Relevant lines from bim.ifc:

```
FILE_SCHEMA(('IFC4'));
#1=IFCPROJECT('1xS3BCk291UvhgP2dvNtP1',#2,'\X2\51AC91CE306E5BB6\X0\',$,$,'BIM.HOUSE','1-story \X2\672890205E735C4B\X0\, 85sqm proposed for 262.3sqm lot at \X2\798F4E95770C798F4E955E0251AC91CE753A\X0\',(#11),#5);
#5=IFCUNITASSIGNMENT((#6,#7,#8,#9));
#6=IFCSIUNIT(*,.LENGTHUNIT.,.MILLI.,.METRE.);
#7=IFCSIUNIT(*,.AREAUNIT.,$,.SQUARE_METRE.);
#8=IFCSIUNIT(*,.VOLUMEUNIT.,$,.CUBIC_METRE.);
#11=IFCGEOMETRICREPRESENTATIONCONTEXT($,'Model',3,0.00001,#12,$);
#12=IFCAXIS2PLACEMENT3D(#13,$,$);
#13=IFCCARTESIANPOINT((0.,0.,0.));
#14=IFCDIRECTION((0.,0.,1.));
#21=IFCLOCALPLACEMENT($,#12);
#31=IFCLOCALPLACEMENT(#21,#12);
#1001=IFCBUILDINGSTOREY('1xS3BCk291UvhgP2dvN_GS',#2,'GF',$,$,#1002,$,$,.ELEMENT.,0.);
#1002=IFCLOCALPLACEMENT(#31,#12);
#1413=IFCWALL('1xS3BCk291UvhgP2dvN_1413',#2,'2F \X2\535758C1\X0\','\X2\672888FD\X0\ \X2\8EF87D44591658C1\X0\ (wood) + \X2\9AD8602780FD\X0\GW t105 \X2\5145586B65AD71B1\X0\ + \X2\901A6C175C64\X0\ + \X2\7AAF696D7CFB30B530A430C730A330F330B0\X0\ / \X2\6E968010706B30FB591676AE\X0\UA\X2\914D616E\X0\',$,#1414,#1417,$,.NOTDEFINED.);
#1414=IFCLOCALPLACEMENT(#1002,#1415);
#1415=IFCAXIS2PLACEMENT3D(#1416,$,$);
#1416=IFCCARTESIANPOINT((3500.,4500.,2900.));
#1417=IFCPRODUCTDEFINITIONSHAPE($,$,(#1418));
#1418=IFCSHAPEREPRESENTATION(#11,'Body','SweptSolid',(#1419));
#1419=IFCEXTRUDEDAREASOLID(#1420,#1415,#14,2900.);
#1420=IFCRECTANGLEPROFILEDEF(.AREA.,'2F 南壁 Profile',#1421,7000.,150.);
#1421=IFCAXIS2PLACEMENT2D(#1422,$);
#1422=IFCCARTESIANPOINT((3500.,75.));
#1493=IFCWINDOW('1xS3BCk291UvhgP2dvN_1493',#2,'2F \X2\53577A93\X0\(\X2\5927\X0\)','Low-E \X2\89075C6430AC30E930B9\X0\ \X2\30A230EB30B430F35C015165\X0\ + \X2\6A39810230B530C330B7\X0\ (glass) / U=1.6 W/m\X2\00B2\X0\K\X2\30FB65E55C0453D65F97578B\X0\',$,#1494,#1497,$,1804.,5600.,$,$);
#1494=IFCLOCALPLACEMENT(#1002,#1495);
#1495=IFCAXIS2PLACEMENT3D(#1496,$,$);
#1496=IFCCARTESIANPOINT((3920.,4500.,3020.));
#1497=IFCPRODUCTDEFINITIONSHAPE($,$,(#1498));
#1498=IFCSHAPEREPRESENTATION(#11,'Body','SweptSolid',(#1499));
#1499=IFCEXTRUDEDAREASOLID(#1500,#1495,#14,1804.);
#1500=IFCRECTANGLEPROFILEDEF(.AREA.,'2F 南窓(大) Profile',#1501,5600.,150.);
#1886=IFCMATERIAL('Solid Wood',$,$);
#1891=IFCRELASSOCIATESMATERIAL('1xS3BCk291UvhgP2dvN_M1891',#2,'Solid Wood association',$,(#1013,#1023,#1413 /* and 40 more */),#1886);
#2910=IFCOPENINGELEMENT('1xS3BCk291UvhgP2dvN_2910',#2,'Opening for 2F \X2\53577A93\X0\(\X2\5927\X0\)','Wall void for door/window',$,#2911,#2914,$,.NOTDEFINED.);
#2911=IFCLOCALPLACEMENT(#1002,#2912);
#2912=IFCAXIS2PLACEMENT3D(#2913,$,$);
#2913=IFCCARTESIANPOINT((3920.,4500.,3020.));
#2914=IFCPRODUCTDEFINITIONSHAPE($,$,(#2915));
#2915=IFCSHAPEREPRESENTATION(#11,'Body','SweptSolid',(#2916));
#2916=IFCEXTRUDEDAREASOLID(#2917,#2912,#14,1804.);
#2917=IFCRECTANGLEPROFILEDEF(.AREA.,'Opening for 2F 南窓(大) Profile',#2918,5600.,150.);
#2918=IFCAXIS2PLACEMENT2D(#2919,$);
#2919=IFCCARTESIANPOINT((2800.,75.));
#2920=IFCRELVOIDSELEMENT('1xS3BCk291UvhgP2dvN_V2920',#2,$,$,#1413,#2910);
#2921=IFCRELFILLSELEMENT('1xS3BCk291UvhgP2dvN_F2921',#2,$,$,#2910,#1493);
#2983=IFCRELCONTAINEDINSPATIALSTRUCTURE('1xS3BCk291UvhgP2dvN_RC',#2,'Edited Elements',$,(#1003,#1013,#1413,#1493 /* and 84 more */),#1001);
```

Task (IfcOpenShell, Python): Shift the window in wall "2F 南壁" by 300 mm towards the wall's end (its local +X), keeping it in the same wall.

```python
import ifcopenshell
import ifcopenshell.api.geometry
import ifcopenshell.util.placement
import ifcopenshell.util.unit

model = ifcopenshell.open("bim.ifc")
unit_scale = ifcopenshell.util.unit.calculate_unit_scale(model)

window = model.by_guid("1xS3BCk291UvhgP2dvN_1493")
opening = window.FillsVoids[0].RelatingOpeningElement
wall = opening.VoidsElements[0].RelatingBuildingElement

wall_matrix = ifcopenshell.util.placement.get_local_placement(wall.ObjectPlacement)
shift = wall_matrix[:3, 0] * 0.3 / unit_scale
before = ifcopenshell.util.placement.get_local_placement(window.ObjectPlacement)[:3, 3].copy()

# The window is not placed relative to its opening, so move both.
for product in (opening, window):
    matrix = ifcopenshell.util.placement.get_local_placement(product.ObjectPlacement)
    matrix[:3, 3] += shift
    ifcopenshell.api.geometry.edit_object_placement(model, product=product, matrix=matrix, is_si=False)

after = ifcopenshell.util.placement.get_local_placement(window.ObjectPlacement)[:3, 3]
print("window moved by", (after - before).round(3) + 0.0)

model.write("bim_edited.ifc")
```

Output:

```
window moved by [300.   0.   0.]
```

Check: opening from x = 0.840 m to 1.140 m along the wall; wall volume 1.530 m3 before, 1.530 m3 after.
